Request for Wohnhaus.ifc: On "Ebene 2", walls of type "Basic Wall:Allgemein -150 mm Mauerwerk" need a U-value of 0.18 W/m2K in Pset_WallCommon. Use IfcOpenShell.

First a look at what the model holds.

```python
import ifcopenshell
import ifcopenshell.util.element

model = ifcopenshell.open("Wohnhaus.ifc")
print(model.schema)
storey = next(s for s in model.by_type("IfcBuildingStorey") if s.Name == "Ebene 2")
walls = [e for e in ifcopenshell.util.element.get_decomposition(storey) if e.is_a("IfcWall")]
seen = {}
for e in walls:
    element_type = ifcopenshell.util.element.get_type(e)
    key = (element_type.Name if element_type != e and element_type else None, ifcopenshell.util.element.get_pset(e, "Pset_WallCommon", "ThermalTransmittance"))
    seen[key] = seen.get(key, 0) + 1
for (name, value), count in sorted(seen.items(), key=str):
    print(count, "x", name, "|", value)
```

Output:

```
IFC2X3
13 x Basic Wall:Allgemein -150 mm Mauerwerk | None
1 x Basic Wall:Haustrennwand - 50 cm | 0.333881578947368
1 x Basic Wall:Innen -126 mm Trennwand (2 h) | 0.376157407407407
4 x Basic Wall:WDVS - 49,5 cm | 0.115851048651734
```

```python
import ifcopenshell
import ifcopenshell.api.pset
import ifcopenshell.util.element

model = ifcopenshell.open("Wohnhaus.ifc")

storey = next(s for s in model.by_type("IfcBuildingStorey") if s.Name == "Ebene 2")
walls = [e for e in ifcopenshell.util.element.get_decomposition(storey) if e.is_a("IfcWall")]

count = 0
for e in walls:
    element_type = ifcopenshell.util.element.get_type(e)
    if element_type in (None, e) or element_type.Name != "Basic Wall:Allgemein -150 mm Mauerwerk":
        continue
    # add_pset returns the element's existing set when there is one.
    pset = ifcopenshell.api.pset.add_pset(model, product=e, name="Pset_WallCommon")
    ifcopenshell.api.pset.edit_pset(model, pset=pset, properties={"ThermalTransmittance": 0.18})
    count += 1

print(count, "walls updated")

model.write("Wohnhaus-out.ifc")
```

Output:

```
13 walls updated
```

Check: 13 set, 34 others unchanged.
